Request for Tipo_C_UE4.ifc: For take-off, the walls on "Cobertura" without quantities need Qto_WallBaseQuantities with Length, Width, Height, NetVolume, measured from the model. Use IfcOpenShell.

First a look at what the model holds.

```python
import ifcopenshell
import ifcopenshell.util.element
import ifcopenshell.util.unit

model = ifcopenshell.open("Tipo_C_UE4.ifc")
print(model.schema)
for unit_type in ("LENGTHUNIT", "AREAUNIT", "VOLUMEUNIT"):
    print(unit_type, ifcopenshell.util.unit.calculate_unit_scale(model, unit_type))
storey = next(s for s in model.by_type("IfcBuildingStorey") if s.Name == "Cobertura")
walls = [e for e in ifcopenshell.util.element.get_decomposition(storey) if e.is_a("IfcWall")]
for e in sorted(walls, key=lambda e: e.id()):
    print(e.id(), e.is_a(), e.Name, list(ifcopenshell.util.element.get_psets(e, qtos_only=True)), sep=" | ")
```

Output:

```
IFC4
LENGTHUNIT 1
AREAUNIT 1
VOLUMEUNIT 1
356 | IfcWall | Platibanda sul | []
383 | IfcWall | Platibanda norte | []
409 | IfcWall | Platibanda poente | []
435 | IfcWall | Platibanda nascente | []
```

```python
import ifcopenshell
import ifcopenshell.api.pset
import ifcopenshell.geom
import ifcopenshell.util.element
import ifcopenshell.util.shape
import ifcopenshell.util.unit

model = ifcopenshell.open("Tipo_C_UE4.ifc")
unit_scale = ifcopenshell.util.unit.calculate_unit_scale(model)
volume_scale = ifcopenshell.util.unit.calculate_unit_scale(model, "VOLUMEUNIT")
settings = ifcopenshell.geom.settings()

storey = next(s for s in model.by_type("IfcBuildingStorey") if s.Name == "Cobertura")
walls = [e for e in ifcopenshell.util.element.get_decomposition(storey) if e.is_a("IfcWall")]

for e in sorted(walls, key=lambda e: e.id()):
    if ifcopenshell.util.element.get_psets(e, qtos_only=True, should_inherit=False):
        continue
    # Geometry comes back in metres, in the element's own axes.
    shape = ifcopenshell.geom.create_shape(settings, e)
    values = {
        "Length": ifcopenshell.util.shape.get_x(shape.geometry) / unit_scale,
        "Width": ifcopenshell.util.shape.get_y(shape.geometry) / unit_scale,
        "Height": ifcopenshell.util.shape.get_z(shape.geometry) / unit_scale,
        "NetVolume": ifcopenshell.util.shape.get_volume(shape.geometry) / volume_scale,
    }
    qto = ifcopenshell.api.pset.add_qto(model, product=e, name="Qto_WallBaseQuantities")
    ifcopenshell.api.pset.edit_qto(model, qto=qto, properties=values)
    print(e.id(), {k: round(v, 3) for k, v in values.items()})

model.write("Tipo_C_UE4_updated.ifc")
```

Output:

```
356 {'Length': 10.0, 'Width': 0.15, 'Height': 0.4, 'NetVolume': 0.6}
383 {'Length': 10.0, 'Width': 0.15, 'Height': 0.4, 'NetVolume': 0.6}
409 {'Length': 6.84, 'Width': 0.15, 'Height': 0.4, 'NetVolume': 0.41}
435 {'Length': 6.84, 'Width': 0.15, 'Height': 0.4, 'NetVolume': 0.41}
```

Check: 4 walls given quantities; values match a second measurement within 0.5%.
